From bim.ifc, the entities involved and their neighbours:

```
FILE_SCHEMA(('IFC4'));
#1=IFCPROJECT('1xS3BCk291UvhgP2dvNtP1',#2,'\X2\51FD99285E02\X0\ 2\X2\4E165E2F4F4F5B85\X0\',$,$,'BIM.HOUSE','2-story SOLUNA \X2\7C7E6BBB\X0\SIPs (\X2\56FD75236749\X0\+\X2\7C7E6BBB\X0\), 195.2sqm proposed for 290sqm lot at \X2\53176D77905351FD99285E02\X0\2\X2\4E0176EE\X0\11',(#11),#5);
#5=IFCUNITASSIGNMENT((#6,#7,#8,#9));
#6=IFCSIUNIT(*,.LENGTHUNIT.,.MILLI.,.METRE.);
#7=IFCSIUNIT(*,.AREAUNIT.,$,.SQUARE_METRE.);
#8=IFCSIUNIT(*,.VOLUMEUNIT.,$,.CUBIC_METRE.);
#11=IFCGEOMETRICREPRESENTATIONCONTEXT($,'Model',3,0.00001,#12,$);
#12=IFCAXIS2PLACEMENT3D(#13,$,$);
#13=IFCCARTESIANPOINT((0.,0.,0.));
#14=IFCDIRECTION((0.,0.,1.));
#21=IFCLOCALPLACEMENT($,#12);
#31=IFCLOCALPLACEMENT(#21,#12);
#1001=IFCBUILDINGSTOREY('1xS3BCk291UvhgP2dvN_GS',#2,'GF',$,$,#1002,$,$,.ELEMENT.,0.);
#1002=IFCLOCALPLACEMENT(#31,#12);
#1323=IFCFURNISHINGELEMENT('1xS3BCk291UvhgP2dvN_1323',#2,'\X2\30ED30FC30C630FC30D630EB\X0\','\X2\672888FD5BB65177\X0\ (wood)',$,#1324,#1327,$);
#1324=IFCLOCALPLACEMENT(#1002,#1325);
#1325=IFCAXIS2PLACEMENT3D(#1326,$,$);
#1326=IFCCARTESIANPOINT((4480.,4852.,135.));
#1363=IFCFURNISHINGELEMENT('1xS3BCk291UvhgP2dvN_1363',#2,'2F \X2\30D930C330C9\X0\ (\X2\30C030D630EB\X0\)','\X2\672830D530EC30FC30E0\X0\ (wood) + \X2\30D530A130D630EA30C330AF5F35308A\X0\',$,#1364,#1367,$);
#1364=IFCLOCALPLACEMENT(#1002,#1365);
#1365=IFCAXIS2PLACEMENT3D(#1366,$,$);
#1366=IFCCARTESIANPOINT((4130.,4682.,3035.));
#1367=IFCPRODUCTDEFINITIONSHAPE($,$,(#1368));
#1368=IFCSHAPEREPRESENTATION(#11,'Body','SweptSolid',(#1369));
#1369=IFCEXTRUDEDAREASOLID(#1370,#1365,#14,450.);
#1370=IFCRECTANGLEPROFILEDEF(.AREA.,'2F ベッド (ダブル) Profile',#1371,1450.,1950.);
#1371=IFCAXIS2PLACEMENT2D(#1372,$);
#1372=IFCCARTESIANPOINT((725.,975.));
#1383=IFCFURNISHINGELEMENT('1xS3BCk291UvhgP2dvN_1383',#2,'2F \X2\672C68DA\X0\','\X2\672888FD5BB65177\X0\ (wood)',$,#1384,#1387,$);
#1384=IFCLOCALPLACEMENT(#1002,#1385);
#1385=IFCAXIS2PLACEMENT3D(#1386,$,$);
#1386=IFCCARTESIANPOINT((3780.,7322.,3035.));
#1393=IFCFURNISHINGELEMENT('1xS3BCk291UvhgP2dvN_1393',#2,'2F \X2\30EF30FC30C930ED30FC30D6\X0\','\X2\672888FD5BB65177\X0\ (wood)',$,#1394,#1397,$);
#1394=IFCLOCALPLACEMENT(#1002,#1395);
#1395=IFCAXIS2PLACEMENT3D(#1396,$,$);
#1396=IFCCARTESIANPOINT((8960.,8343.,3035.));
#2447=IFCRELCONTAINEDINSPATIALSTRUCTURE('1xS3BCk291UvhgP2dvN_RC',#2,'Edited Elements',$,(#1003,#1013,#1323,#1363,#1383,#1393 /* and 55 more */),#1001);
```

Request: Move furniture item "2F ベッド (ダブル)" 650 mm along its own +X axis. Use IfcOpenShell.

```python
import ifcopenshell
import ifcopenshell.api.geometry
import ifcopenshell.util.placement
import ifcopenshell.util.unit

model = ifcopenshell.open("bim.ifc")
unit_scale = ifcopenshell.util.unit.calculate_unit_scale(model)

item = model.by_guid("1xS3BCk291UvhgP2dvN_1363")
matrix = ifcopenshell.util.placement.get_local_placement(item.ObjectPlacement)
matrix[:3, 3] += matrix[:3, 0] * 0.65 / unit_scale
ifcopenshell.api.geometry.edit_object_placement(model, product=item, matrix=matrix, is_si=False)

print(ifcopenshell.util.placement.get_local_placement(item.ObjectPlacement).round(3) + 0.0)

model.write("bim_edited.ifc")
```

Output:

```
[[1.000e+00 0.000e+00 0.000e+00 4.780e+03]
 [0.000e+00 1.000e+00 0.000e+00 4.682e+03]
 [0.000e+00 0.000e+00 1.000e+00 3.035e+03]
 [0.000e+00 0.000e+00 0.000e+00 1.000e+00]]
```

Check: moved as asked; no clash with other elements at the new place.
